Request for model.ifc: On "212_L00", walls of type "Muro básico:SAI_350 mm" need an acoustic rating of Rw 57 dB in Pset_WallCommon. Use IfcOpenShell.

First a look at what the model holds.

```python
import ifcopenshell
import ifcopenshell.util.element

model = ifcopenshell.open("model.ifc")
print(model.schema)
storey = next(s for s in model.by_type("IfcBuildingStorey") if s.Name == "212_L00")
walls = [e for e in ifcopenshell.util.element.get_decomposition(storey) if e.is_a("IfcWall")]
seen = {}
for e in walls:
    element_type = ifcopenshell.util.element.get_type(e)
    key = (element_type.Name if element_type != e and element_type else None, ifcopenshell.util.element.get_pset(e, "Pset_WallCommon", "AcousticRating"))
    seen[key] = seen.get(key, 0) + 1
for (name, value), count in sorted(seen.items(), key=str):
    print(count, "x", name, "|", value)
```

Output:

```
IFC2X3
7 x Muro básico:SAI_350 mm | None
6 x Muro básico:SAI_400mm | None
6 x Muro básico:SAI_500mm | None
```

```python
import ifcopenshell
import ifcopenshell.api.pset
import ifcopenshell.util.element

model = ifcopenshell.open("model.ifc")

storey = next(s for s in model.by_type("IfcBuildingStorey") if s.Name == "212_L00")
walls = [e for e in ifcopenshell.util.element.get_decomposition(storey) if e.is_a("IfcWall")]

count = 0
for e in walls:
    element_type = ifcopenshell.util.element.get_type(e)
    if element_type in (None, e) or element_type.Name != "Muro básico:SAI_350 mm":
        continue
    # add_pset returns the element's existing set when there is one.
    pset = ifcopenshell.api.pset.add_pset(model, product=e, name="Pset_WallCommon")
    ifcopenshell.api.pset.edit_pset(model, pset=pset, properties={"AcousticRating": "Rw 57 dB"})
    count += 1

print(count, "walls updated")

model.write("model_updated.ifc")
```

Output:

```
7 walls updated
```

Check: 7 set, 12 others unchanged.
